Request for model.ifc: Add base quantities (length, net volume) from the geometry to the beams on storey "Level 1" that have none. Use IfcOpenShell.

First a look at what the model holds.

```python
import ifcopenshell
import ifcopenshell.util.element
import ifcopenshell.util.unit

model = ifcopenshell.open("model.ifc")
print(model.schema)
for unit_type in ("LENGTHUNIT", "AREAUNIT", "VOLUMEUNIT"):
    print(unit_type, ifcopenshell.util.unit.calculate_unit_scale(model, unit_type))
storey = next(s for s in model.by_type("IfcBuildingStorey") if s.Name == "Level 1")
beams = [e for e in ifcopenshell.util.element.get_decomposition(storey) if e.is_a("IfcBeam")]
for e in sorted(beams, key=lambda e: e.id()):
    print(e.id(), e.is_a(), e.Name, list(ifcopenshell.util.element.get_psets(e, qtos_only=True)), sep=" | ")
```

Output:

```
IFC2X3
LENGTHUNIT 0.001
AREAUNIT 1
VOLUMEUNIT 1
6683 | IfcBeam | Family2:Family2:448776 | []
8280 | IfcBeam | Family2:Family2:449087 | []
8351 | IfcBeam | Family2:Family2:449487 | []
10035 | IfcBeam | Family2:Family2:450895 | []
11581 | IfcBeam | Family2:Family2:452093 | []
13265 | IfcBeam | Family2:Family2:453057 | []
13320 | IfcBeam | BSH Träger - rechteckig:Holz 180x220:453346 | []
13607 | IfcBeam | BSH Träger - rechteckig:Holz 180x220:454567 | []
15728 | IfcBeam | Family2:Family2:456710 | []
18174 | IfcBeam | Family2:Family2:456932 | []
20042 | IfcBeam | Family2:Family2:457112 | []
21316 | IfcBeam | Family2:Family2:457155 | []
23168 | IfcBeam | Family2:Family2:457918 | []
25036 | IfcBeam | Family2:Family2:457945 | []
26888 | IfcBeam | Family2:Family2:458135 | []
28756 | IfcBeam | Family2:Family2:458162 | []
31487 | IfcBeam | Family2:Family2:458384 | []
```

```python
import ifcopenshell
import ifcopenshell.api.pset
import ifcopenshell.geom
import ifcopenshell.util.element
import ifcopenshell.util.shape
import ifcopenshell.util.unit

model = ifcopenshell.open("model.ifc")
unit_scale = ifcopenshell.util.unit.calculate_unit_scale(model)
volume_scale = ifcopenshell.util.unit.calculate_unit_scale(model, "VOLUMEUNIT")
settings = ifcopenshell.geom.settings()

storey = next(s for s in model.by_type("IfcBuildingStorey") if s.Name == "Level 1")
beams = [e for e in ifcopenshell.util.element.get_decomposition(storey) if e.is_a("IfcBeam")]

for e in sorted(beams, key=lambda e: e.id()):
    if ifcopenshell.util.element.get_psets(e, qtos_only=True, should_inherit=False):
        continue
    # Geometry comes back in metres, in the element's own axes.
    shape = ifcopenshell.geom.create_shape(settings, e)
    values = {
        "Length": ifcopenshell.util.shape.get_max_xyz(shape.geometry) / unit_scale,
        "NetVolume": ifcopenshell.util.shape.get_volume(shape.geometry) / volume_scale,
    }
    qto = ifcopenshell.api.pset.add_qto(model, product=e, name="BaseQuantities")
    ifcopenshell.api.pset.edit_qto(model, qto=qto, properties=values)
    print(e.id(), {k: round(v, 3) for k, v in values.items()})

model.write("model_v2.ifc")
```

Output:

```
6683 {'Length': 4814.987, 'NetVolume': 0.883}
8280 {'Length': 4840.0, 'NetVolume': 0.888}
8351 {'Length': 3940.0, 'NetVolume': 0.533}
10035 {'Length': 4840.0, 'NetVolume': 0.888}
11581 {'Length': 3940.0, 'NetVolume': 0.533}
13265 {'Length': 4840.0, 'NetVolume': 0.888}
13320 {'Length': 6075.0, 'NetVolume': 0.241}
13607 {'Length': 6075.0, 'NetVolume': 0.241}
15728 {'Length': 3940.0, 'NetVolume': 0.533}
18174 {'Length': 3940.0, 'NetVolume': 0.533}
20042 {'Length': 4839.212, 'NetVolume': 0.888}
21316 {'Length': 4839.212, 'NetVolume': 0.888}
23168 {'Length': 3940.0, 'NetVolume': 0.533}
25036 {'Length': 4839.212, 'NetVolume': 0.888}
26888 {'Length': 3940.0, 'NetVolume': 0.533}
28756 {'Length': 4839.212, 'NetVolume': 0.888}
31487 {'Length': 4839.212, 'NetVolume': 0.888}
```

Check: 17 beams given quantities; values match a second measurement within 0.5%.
